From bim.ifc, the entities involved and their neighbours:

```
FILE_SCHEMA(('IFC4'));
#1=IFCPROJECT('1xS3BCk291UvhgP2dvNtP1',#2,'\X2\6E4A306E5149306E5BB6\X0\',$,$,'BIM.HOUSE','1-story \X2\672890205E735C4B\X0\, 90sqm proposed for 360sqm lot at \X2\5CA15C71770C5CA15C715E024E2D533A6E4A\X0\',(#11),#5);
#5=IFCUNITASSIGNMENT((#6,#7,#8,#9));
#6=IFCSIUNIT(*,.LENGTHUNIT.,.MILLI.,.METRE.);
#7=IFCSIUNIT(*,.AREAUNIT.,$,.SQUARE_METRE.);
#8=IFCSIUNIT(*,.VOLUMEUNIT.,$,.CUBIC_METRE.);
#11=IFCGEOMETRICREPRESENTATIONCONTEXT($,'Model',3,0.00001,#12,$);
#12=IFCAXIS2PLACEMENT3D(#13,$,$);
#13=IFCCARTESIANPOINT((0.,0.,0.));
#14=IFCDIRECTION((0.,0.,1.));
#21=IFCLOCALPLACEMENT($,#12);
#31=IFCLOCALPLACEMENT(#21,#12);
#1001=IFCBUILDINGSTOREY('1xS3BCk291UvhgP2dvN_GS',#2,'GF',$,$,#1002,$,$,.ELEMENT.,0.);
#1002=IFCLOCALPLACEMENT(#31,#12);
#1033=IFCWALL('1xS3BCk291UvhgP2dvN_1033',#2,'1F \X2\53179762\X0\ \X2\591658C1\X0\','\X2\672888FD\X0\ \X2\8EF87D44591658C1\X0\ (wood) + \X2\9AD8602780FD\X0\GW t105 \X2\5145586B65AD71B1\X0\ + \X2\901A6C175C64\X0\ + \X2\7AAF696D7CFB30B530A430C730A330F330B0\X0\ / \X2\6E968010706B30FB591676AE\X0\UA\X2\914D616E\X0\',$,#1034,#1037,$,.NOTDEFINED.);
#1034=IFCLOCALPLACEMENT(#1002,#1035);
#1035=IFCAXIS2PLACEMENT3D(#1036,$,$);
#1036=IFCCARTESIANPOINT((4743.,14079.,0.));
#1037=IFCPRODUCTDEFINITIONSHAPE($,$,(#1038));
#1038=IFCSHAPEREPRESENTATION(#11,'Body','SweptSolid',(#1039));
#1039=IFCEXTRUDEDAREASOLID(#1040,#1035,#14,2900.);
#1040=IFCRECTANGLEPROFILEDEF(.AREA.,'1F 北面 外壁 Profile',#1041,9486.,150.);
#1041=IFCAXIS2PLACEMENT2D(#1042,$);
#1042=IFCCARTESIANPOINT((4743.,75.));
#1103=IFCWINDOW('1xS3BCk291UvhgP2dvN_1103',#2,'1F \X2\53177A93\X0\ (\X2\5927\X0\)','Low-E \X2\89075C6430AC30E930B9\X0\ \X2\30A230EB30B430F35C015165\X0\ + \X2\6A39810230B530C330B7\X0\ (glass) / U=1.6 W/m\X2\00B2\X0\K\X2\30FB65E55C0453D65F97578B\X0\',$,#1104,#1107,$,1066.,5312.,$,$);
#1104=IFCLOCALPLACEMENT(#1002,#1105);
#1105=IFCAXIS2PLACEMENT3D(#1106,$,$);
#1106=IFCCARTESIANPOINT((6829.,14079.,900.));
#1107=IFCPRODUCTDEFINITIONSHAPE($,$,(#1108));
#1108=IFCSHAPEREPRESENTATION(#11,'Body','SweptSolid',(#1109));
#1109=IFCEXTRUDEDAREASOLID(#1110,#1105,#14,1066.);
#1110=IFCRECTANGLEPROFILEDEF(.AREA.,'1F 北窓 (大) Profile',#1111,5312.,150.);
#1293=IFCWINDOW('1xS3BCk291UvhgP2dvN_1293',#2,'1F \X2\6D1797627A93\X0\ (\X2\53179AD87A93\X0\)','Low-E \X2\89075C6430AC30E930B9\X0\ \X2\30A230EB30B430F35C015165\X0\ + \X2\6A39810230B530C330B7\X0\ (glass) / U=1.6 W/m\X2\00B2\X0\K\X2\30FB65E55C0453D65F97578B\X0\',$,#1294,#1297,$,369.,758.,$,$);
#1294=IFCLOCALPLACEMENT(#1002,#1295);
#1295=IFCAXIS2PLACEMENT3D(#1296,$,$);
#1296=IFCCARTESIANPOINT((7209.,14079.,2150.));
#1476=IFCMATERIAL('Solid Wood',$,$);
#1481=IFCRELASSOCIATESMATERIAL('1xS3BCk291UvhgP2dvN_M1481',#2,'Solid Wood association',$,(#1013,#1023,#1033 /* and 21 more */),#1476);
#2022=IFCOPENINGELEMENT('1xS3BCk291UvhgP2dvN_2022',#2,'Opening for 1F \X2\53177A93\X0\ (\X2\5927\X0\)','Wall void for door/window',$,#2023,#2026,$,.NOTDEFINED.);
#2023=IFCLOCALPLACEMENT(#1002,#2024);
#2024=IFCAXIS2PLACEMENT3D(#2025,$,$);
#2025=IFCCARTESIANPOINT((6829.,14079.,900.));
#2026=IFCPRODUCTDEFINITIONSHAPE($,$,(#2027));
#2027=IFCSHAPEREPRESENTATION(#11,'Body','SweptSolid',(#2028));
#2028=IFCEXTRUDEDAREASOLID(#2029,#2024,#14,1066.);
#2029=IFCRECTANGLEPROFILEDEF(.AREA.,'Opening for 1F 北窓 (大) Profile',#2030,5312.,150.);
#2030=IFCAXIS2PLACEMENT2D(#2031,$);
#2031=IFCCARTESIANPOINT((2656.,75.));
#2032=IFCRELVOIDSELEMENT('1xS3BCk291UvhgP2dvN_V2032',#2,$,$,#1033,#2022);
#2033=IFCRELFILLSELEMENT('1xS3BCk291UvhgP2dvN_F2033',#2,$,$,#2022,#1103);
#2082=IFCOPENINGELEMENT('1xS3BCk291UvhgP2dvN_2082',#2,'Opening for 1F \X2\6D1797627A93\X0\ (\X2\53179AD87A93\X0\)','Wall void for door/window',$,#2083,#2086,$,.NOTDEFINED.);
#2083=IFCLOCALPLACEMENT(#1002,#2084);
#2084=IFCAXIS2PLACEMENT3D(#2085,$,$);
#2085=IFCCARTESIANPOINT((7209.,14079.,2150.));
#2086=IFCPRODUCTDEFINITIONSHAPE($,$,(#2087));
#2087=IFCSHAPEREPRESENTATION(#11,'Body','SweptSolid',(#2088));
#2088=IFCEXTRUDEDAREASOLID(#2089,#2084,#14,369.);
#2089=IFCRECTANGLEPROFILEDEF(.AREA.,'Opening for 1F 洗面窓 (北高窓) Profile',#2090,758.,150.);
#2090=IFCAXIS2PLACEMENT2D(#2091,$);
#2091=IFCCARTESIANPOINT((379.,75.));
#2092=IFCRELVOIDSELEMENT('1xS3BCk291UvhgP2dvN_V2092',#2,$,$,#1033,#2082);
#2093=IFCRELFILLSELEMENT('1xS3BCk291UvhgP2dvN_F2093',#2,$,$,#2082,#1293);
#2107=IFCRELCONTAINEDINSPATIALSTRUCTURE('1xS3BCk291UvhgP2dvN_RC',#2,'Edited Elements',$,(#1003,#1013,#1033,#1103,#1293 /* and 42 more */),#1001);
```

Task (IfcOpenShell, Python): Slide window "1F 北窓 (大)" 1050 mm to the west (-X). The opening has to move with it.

```python
import ifcopenshell
import ifcopenshell.api.geometry
import ifcopenshell.util.placement

model = ifcopenshell.open("bim.ifc")

window = model.by_guid("1xS3BCk291UvhgP2dvN_1103")
opening = window.FillsVoids[0].RelatingOpeningElement
wall = opening.VoidsElements[0].RelatingBuildingElement

wall_matrix = ifcopenshell.util.placement.get_local_placement(wall.ObjectPlacement)
shift = wall_matrix[:3, 0] * -1050.0
before = ifcopenshell.util.placement.get_local_placement(window.ObjectPlacement)[:3, 3].copy()

# The window is not placed relative to its opening, so move both.
for product in (opening, window):
    matrix = ifcopenshell.util.placement.get_local_placement(product.ObjectPlacement)
    matrix[:3, 3] += shift
    ifcopenshell.api.geometry.edit_object_placement(model, product=product, matrix=matrix, is_si=False)

after = ifcopenshell.util.placement.get_local_placement(window.ObjectPlacement)[:3, 3]
print("window moved by", (after - before).round(3) + 0.0)

model.write("bim_updated.ifc")
```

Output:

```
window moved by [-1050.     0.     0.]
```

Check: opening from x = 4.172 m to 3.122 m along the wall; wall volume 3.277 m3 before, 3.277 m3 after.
